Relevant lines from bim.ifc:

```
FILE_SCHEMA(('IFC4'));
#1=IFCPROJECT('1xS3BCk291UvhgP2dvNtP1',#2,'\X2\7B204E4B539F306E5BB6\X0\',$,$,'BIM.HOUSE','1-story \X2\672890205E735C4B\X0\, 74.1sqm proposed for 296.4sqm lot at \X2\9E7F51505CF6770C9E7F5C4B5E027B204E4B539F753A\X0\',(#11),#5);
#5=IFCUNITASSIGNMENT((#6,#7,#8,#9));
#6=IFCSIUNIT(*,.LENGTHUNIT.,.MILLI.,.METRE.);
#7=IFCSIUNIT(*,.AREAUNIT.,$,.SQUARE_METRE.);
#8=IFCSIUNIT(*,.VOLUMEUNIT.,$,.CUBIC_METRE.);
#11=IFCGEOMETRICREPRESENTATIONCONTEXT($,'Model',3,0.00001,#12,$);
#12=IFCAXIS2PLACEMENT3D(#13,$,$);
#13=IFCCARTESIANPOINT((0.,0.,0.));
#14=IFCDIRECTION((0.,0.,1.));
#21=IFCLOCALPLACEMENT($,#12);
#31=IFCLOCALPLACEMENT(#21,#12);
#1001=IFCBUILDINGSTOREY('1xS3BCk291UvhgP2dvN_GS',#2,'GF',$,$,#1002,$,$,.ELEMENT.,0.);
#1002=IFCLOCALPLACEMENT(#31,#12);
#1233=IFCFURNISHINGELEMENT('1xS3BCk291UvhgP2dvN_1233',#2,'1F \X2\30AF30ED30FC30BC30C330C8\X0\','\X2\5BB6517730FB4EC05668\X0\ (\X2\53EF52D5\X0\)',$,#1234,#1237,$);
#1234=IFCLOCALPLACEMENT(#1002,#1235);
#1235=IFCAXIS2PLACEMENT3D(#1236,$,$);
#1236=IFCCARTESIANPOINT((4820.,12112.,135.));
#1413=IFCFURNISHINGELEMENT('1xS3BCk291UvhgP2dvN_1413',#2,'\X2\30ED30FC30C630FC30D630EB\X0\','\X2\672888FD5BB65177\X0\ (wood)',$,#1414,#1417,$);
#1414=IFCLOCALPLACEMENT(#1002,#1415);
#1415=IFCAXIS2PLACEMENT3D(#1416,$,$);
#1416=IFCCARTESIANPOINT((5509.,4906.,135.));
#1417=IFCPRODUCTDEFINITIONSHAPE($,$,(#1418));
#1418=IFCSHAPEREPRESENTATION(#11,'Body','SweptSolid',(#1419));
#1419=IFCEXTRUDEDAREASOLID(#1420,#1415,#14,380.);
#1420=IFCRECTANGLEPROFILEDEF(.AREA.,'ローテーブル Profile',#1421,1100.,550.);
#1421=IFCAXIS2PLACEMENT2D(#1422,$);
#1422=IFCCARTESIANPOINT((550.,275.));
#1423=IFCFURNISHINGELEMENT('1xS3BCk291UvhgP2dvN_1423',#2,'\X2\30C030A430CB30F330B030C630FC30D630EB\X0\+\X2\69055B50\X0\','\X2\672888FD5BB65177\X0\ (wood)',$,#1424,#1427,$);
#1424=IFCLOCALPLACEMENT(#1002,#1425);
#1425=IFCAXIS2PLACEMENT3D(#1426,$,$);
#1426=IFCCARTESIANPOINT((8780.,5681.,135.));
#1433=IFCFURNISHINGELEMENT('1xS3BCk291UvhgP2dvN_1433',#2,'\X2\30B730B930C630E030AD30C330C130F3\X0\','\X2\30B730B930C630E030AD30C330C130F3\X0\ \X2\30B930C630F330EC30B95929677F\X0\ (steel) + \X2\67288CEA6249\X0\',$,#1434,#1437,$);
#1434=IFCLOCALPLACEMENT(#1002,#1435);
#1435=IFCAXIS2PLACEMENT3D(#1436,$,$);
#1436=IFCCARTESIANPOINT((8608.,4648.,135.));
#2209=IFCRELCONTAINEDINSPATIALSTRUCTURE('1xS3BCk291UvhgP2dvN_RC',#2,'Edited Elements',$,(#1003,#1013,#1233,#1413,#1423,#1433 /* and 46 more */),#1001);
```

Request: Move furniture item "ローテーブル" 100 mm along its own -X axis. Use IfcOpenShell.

```python
import ifcopenshell
import ifcopenshell.api.geometry
import ifcopenshell.util.placement
import ifcopenshell.util.unit

model = ifcopenshell.open("bim.ifc")
unit_scale = ifcopenshell.util.unit.calculate_unit_scale(model)

item = model.by_guid("1xS3BCk291UvhgP2dvN_1413")
matrix = ifcopenshell.util.placement.get_local_placement(item.ObjectPlacement)
matrix[:3, 3] -= matrix[:3, 0] * 0.1 / unit_scale
ifcopenshell.api.geometry.edit_object_placement(model, product=item, matrix=matrix, is_si=False)

print(ifcopenshell.util.placement.get_local_placement(item.ObjectPlacement).round(3) + 0.0)

model.write("bim_rev.ifc")
```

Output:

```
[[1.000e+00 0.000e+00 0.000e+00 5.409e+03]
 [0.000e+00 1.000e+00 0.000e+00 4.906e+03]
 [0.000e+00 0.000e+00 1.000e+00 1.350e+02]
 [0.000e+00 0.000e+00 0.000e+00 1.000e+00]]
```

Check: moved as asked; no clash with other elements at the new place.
